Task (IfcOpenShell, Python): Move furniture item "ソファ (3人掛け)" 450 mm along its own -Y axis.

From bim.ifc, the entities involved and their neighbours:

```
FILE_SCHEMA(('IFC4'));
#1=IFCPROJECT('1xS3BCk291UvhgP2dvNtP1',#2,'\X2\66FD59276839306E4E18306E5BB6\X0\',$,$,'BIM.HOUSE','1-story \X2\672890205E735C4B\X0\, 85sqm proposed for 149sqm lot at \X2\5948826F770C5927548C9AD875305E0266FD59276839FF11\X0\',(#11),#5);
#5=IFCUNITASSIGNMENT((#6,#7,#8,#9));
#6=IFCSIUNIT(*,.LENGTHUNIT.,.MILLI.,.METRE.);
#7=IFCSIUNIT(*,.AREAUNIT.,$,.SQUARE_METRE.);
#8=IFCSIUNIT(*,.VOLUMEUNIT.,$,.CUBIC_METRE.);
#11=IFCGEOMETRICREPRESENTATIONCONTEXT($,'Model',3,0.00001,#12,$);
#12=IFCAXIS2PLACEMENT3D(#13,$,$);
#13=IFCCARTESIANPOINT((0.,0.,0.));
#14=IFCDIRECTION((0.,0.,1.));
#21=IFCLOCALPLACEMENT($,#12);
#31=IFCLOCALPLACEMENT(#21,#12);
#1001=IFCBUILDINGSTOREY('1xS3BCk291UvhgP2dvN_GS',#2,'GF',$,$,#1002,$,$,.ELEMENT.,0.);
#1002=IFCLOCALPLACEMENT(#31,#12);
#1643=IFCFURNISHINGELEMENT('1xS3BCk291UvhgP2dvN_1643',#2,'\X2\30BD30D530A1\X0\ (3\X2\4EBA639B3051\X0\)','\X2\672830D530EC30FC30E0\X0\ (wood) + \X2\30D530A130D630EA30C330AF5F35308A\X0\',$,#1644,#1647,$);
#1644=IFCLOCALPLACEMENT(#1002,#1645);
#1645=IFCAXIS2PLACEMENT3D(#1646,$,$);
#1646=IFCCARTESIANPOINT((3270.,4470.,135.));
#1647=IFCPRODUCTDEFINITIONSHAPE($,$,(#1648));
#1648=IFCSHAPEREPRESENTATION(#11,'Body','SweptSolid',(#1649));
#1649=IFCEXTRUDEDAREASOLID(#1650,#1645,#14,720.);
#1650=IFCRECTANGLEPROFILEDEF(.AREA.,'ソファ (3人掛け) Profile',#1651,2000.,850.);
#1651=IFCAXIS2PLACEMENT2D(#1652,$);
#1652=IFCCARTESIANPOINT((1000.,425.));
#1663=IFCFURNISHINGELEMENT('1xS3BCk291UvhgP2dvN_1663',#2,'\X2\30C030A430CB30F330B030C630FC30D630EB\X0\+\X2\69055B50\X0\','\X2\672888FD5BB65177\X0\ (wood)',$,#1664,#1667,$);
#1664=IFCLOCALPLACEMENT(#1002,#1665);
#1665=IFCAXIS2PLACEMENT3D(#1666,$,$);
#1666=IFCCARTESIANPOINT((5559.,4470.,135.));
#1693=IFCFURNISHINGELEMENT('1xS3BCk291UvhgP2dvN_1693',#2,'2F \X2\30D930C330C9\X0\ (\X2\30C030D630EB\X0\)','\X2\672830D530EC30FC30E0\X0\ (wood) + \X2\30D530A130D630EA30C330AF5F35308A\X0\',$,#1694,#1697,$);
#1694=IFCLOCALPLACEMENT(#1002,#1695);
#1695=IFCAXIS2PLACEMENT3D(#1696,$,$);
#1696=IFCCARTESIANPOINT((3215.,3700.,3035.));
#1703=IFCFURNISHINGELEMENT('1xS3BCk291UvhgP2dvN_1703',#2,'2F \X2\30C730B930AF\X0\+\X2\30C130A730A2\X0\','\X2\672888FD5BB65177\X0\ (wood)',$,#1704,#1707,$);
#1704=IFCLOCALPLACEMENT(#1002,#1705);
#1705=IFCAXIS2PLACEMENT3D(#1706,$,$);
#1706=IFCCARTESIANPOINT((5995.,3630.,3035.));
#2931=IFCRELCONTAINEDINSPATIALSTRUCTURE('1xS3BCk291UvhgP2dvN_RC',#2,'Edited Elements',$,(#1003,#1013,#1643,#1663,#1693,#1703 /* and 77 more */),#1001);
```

```python
import ifcopenshell
import ifcopenshell.api.geometry
import ifcopenshell.util.placement
import ifcopenshell.util.unit

model = ifcopenshell.open("bim.ifc")
unit_scale = ifcopenshell.util.unit.calculate_unit_scale(model)

item = model.by_id(1643)
matrix = ifcopenshell.util.placement.get_local_placement(item.ObjectPlacement)
matrix[:3, 3] -= matrix[:3, 1] * 0.45 / unit_scale
ifcopenshell.api.geometry.edit_object_placement(model, product=item, matrix=matrix, is_si=False)

print(ifcopenshell.util.placement.get_local_placement(item.ObjectPlacement).round(3) + 0.0)

model.write("bim_rev.ifc")
```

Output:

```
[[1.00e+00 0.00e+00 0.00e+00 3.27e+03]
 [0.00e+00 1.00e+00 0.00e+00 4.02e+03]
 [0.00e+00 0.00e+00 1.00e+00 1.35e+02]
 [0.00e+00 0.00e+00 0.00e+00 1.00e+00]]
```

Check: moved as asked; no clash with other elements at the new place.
